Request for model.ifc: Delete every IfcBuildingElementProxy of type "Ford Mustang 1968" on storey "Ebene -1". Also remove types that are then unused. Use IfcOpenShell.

First a look at what the model holds.

```python
import ifcopenshell
import ifcopenshell.util.element

model = ifcopenshell.open("model.ifc")
print(model.schema)
storey = next(s for s in model.by_type("IfcBuildingStorey") if s.Name == "Ebene -1")
proxies = [e for e in ifcopenshell.util.element.get_decomposition(storey) if e.is_a("IfcBuildingElementProxy")]
seen = {}
for e in proxies:
    element_type = ifcopenshell.util.element.get_type(e)
    name = element_type.Name if element_type not in (None, e) else None
    seen[name] = seen.get(name, 0) + 1
for name, count in sorted(seen.items(), key=str):
    print(count, "x", name)
```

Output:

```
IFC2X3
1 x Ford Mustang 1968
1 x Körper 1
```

```python
import ifcopenshell
import ifcopenshell.api.root
import ifcopenshell.util.element

model = ifcopenshell.open("model.ifc")

storey = next(s for s in model.by_type("IfcBuildingStorey") if s.Name == "Ebene -1")
proxies = [e for e in ifcopenshell.util.element.get_decomposition(storey) if e.is_a("IfcBuildingElementProxy")]
targets = [e for e in proxies if (t := ifcopenshell.util.element.get_type(e)) not in (None, e) and t.Name == "Ford Mustang 1968"]
types = {ifcopenshell.util.element.get_type(e) for e in targets} - {None, *targets}

for e in targets:
    ifcopenshell.api.root.remove_product(model, product=e)
print(len(targets), "removed")

unused = [t for t in types if not ifcopenshell.util.element.get_types(t)]
for t in unused:
    ifcopenshell.api.root.remove_product(model, product=t)
print(len(unused), "unused types removed")

model.write("model_v2.ifc")
```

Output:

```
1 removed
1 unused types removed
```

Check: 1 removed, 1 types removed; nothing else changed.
